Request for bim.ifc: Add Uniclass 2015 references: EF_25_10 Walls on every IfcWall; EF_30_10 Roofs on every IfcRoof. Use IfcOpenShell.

First a look at what the model holds.

```python
import ifcopenshell

model = ifcopenshell.open("bim.ifc")
print(model.schema)
print("classifications:", [c.Name for c in model.by_type("IfcClassification")])
for ifc_class in ("IfcDoor", "IfcRoof", "IfcStair", "IfcWall", "IfcWindow"):
    print(ifc_class, len(model.by_type(ifc_class)))
```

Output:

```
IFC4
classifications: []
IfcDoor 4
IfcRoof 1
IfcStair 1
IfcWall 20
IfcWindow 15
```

```python
import ifcopenshell
import ifcopenshell.api.classification

model = ifcopenshell.open("bim.ifc")

system = ifcopenshell.api.classification.add_classification(model, classification="Uniclass 2015")

codes = {
    "IfcWall": ("EF_25_10", "Walls"),
    "IfcRoof": ("EF_30_10", "Roofs"),
}
for ifc_class, (code, name) in codes.items():
    products = model.by_type(ifc_class)
    ifcopenshell.api.classification.add_reference(
        model, products=products, classification=system, identification=code, name=name
    )
    print(code, len(products))

model.write("bim_v2.ifc")
```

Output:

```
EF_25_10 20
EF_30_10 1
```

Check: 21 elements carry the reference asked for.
